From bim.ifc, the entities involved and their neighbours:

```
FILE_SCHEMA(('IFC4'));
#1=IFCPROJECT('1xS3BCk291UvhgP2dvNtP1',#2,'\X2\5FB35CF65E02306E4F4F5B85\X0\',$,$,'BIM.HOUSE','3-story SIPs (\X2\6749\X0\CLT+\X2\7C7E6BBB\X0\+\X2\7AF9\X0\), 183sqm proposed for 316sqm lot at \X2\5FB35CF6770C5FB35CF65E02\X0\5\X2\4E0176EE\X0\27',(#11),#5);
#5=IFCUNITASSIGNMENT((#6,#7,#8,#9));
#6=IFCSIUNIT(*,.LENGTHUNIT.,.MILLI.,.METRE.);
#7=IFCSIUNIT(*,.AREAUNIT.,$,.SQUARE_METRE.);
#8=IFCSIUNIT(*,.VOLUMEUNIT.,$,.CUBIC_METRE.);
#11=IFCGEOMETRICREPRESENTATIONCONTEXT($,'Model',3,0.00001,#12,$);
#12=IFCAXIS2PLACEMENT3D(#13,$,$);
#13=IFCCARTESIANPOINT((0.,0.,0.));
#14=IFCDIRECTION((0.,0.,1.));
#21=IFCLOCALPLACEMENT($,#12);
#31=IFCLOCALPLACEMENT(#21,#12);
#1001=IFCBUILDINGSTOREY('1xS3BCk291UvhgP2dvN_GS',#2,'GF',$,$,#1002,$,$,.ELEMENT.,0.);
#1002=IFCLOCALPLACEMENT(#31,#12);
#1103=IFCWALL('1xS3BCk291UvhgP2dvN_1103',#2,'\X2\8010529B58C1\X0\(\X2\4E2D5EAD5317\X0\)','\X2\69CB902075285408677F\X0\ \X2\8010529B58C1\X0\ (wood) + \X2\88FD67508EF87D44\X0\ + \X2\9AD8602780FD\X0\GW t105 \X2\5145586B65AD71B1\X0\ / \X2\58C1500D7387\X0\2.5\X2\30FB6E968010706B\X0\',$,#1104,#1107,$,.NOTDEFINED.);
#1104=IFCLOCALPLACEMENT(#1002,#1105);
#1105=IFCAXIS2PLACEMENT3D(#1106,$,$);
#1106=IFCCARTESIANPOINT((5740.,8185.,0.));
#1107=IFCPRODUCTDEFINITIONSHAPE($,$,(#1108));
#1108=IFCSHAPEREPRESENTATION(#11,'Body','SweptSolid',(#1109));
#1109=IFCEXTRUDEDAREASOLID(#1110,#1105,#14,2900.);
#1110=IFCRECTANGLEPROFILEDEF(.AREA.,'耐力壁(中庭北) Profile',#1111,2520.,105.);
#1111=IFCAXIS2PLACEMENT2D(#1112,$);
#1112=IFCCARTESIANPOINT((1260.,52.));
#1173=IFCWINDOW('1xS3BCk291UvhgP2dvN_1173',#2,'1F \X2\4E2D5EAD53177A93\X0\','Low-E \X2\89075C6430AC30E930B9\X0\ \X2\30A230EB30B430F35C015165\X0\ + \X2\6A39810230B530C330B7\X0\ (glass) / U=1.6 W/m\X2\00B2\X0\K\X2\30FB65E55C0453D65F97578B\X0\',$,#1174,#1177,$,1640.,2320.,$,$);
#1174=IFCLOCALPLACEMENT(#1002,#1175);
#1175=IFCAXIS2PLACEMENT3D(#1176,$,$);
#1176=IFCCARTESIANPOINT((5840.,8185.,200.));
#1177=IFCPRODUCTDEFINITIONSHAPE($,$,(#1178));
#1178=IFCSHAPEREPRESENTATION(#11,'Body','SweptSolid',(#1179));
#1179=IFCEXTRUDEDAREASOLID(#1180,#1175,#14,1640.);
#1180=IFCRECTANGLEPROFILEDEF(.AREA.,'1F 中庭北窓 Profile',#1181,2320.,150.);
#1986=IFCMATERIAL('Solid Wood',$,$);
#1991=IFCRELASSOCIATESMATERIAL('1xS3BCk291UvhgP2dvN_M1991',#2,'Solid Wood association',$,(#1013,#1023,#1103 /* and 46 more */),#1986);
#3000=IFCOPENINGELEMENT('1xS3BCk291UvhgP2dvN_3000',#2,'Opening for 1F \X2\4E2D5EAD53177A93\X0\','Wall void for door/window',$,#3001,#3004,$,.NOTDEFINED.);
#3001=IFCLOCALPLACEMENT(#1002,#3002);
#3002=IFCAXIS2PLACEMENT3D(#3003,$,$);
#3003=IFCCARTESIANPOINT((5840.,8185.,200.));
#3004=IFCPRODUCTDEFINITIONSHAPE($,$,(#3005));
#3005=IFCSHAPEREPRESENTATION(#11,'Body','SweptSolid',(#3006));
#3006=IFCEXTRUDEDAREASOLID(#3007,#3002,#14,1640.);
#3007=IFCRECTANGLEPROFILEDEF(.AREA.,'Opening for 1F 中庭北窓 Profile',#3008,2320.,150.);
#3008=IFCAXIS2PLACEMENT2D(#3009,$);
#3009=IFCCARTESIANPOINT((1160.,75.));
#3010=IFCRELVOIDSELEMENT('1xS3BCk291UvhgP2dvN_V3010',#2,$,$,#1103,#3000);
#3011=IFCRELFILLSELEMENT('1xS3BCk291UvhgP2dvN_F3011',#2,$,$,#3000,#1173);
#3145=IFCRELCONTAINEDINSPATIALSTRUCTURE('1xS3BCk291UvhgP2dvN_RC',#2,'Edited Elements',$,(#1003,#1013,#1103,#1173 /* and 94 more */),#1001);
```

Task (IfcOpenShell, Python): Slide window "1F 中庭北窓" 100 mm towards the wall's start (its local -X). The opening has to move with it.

```python
import ifcopenshell
import ifcopenshell.api.geometry
import ifcopenshell.util.placement

model = ifcopenshell.open("bim.ifc")

window = model.by_id(1173)
opening = window.FillsVoids[0].RelatingOpeningElement
wall = opening.VoidsElements[0].RelatingBuildingElement

wall_matrix = ifcopenshell.util.placement.get_local_placement(wall.ObjectPlacement)
shift = wall_matrix[:3, 0] * -100.0
before = ifcopenshell.util.placement.get_local_placement(window.ObjectPlacement)[:3, 3].copy()

# The window is not placed relative to its opening, so move both.
for product in (opening, window):
    matrix = ifcopenshell.util.placement.get_local_placement(product.ObjectPlacement)
    matrix[:3, 3] += shift
    ifcopenshell.api.geometry.edit_object_placement(model, product=product, matrix=matrix, is_si=False)

after = ifcopenshell.util.placement.get_local_placement(window.ObjectPlacement)[:3, 3]
print("window moved by", (after - before).round(3) + 0.0)

model.write("bim-out.ifc")
```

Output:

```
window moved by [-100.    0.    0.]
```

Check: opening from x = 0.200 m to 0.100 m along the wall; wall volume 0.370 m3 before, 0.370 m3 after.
